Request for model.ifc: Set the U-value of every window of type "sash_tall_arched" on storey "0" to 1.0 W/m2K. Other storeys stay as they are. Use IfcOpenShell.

First a look at what the model holds.

```python
import ifcopenshell
import ifcopenshell.util.element

model = ifcopenshell.open("model.ifc")
print(model.schema)
storey = next(s for s in model.by_type("IfcBuildingStorey") if s.Name == "0")
windows = [e for e in ifcopenshell.util.element.get_decomposition(storey) if e.is_a("IfcWindow")]
seen = {}
for e in windows:
    element_type = ifcopenshell.util.element.get_type(e)
    key = (element_type.Name if element_type != e and element_type else None, ifcopenshell.util.element.get_pset(e, "Pset_WindowCommon", "ThermalTransmittance"))
    seen[key] = seen.get(key, 0) + 1
for (name, value), count in sorted(seen.items(), key=str):
    print(count, "x", name, "|", value)
```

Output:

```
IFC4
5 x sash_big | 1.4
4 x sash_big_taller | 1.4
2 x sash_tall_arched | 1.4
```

```python
import ifcopenshell
import ifcopenshell.api.pset
import ifcopenshell.util.element

model = ifcopenshell.open("model.ifc")

storey = next(s for s in model.by_type("IfcBuildingStorey") if s.Name == "0")
windows = [e for e in ifcopenshell.util.element.get_decomposition(storey) if e.is_a("IfcWindow")]

count = 0
for e in windows:
    element_type = ifcopenshell.util.element.get_type(e)
    if element_type in (None, e) or element_type.Name != "sash_tall_arched":
        continue
    # add_pset returns the element's existing set when there is one.
    pset = ifcopenshell.api.pset.add_pset(model, product=e, name="Pset_WindowCommon")
    ifcopenshell.api.pset.edit_pset(model, pset=pset, properties={"ThermalTransmittance": 1.0})
    count += 1

print(count, "windows updated")

model.write("model_edited.ifc")
```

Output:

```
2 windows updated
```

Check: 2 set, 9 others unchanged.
